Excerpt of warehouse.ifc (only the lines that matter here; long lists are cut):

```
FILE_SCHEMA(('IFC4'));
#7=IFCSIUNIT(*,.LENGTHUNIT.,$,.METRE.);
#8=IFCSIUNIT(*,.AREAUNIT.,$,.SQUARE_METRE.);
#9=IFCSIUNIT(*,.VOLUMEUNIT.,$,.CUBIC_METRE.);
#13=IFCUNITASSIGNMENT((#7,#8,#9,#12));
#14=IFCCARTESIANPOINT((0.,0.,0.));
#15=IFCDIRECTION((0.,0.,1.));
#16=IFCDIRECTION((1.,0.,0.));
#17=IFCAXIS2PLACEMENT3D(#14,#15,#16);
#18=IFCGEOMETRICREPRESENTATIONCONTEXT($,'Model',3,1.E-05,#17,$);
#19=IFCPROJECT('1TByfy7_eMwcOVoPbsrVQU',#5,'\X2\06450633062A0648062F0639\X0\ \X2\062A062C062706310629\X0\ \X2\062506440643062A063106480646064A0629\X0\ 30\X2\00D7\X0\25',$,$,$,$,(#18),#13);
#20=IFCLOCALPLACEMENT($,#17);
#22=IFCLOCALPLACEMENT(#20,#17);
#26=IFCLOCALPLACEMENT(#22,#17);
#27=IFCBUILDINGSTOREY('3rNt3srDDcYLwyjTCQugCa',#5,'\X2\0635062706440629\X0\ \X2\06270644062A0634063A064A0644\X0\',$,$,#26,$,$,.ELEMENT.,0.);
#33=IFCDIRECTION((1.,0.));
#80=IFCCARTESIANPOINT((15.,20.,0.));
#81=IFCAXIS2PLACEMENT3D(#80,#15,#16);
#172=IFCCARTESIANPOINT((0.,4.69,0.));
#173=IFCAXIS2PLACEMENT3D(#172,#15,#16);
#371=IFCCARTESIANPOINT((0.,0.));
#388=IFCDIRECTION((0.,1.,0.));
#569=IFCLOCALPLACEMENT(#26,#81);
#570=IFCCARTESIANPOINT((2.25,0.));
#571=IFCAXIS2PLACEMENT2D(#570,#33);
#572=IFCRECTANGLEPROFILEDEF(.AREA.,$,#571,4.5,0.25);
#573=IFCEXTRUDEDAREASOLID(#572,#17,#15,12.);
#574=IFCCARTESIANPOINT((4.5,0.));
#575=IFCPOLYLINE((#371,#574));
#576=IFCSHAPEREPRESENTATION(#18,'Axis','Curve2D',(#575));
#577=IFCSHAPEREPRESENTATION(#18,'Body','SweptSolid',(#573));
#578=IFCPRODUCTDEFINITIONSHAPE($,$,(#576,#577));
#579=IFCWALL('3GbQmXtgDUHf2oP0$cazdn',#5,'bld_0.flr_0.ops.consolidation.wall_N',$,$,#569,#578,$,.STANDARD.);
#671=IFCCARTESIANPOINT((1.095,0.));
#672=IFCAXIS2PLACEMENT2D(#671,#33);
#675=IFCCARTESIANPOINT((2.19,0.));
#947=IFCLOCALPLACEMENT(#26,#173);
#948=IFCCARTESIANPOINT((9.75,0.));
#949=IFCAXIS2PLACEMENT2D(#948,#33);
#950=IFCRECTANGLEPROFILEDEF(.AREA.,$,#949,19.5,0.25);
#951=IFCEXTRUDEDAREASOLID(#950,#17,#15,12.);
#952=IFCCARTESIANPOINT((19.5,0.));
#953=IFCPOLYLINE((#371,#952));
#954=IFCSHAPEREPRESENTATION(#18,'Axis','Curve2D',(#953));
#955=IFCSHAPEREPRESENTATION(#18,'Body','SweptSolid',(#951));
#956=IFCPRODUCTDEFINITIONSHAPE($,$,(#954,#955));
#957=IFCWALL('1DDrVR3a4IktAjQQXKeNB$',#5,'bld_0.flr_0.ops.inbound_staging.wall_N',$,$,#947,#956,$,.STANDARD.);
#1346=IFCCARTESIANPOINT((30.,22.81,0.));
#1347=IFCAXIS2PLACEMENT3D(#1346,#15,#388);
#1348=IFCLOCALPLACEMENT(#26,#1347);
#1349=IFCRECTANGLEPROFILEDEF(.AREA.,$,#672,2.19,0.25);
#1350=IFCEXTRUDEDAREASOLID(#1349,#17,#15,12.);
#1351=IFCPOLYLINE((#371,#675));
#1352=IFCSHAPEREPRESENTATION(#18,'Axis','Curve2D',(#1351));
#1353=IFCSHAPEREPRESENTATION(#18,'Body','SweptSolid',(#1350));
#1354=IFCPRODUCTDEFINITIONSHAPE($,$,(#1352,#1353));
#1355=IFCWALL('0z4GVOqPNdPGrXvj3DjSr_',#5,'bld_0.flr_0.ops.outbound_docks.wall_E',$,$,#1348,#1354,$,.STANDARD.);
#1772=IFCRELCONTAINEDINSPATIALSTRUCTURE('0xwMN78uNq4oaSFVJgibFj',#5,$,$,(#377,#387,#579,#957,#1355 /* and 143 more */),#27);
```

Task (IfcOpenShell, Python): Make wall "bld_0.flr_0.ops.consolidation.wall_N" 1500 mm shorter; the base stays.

```python
import ifcopenshell
import ifcopenshell.geom
import ifcopenshell.util.shape

model = ifcopenshell.open("warehouse.ifc")
settings = ifcopenshell.geom.settings()


def volume(element):
    """Net volume in cubic metres, openings subtracted."""
    shape = ifcopenshell.geom.create_shape(settings, element)
    return ifcopenshell.util.shape.get_volume(shape.geometry)


wall = model.by_id(579)
before = volume(wall)

body = next(r for r in wall.Representation.Representations if r.RepresentationIdentifier == "Body")
solid = body.Items[0]
old_height = solid.Depth
solid.Depth -= 1.5
after = volume(wall)

print(f"height {old_height:g} -> {solid.Depth:g}, volume {before:.3f} -> {after:.3f} m3")

model.write("warehouse_rev.ifc")
```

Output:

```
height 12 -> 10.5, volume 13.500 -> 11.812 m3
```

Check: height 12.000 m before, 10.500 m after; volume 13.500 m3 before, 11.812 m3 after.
